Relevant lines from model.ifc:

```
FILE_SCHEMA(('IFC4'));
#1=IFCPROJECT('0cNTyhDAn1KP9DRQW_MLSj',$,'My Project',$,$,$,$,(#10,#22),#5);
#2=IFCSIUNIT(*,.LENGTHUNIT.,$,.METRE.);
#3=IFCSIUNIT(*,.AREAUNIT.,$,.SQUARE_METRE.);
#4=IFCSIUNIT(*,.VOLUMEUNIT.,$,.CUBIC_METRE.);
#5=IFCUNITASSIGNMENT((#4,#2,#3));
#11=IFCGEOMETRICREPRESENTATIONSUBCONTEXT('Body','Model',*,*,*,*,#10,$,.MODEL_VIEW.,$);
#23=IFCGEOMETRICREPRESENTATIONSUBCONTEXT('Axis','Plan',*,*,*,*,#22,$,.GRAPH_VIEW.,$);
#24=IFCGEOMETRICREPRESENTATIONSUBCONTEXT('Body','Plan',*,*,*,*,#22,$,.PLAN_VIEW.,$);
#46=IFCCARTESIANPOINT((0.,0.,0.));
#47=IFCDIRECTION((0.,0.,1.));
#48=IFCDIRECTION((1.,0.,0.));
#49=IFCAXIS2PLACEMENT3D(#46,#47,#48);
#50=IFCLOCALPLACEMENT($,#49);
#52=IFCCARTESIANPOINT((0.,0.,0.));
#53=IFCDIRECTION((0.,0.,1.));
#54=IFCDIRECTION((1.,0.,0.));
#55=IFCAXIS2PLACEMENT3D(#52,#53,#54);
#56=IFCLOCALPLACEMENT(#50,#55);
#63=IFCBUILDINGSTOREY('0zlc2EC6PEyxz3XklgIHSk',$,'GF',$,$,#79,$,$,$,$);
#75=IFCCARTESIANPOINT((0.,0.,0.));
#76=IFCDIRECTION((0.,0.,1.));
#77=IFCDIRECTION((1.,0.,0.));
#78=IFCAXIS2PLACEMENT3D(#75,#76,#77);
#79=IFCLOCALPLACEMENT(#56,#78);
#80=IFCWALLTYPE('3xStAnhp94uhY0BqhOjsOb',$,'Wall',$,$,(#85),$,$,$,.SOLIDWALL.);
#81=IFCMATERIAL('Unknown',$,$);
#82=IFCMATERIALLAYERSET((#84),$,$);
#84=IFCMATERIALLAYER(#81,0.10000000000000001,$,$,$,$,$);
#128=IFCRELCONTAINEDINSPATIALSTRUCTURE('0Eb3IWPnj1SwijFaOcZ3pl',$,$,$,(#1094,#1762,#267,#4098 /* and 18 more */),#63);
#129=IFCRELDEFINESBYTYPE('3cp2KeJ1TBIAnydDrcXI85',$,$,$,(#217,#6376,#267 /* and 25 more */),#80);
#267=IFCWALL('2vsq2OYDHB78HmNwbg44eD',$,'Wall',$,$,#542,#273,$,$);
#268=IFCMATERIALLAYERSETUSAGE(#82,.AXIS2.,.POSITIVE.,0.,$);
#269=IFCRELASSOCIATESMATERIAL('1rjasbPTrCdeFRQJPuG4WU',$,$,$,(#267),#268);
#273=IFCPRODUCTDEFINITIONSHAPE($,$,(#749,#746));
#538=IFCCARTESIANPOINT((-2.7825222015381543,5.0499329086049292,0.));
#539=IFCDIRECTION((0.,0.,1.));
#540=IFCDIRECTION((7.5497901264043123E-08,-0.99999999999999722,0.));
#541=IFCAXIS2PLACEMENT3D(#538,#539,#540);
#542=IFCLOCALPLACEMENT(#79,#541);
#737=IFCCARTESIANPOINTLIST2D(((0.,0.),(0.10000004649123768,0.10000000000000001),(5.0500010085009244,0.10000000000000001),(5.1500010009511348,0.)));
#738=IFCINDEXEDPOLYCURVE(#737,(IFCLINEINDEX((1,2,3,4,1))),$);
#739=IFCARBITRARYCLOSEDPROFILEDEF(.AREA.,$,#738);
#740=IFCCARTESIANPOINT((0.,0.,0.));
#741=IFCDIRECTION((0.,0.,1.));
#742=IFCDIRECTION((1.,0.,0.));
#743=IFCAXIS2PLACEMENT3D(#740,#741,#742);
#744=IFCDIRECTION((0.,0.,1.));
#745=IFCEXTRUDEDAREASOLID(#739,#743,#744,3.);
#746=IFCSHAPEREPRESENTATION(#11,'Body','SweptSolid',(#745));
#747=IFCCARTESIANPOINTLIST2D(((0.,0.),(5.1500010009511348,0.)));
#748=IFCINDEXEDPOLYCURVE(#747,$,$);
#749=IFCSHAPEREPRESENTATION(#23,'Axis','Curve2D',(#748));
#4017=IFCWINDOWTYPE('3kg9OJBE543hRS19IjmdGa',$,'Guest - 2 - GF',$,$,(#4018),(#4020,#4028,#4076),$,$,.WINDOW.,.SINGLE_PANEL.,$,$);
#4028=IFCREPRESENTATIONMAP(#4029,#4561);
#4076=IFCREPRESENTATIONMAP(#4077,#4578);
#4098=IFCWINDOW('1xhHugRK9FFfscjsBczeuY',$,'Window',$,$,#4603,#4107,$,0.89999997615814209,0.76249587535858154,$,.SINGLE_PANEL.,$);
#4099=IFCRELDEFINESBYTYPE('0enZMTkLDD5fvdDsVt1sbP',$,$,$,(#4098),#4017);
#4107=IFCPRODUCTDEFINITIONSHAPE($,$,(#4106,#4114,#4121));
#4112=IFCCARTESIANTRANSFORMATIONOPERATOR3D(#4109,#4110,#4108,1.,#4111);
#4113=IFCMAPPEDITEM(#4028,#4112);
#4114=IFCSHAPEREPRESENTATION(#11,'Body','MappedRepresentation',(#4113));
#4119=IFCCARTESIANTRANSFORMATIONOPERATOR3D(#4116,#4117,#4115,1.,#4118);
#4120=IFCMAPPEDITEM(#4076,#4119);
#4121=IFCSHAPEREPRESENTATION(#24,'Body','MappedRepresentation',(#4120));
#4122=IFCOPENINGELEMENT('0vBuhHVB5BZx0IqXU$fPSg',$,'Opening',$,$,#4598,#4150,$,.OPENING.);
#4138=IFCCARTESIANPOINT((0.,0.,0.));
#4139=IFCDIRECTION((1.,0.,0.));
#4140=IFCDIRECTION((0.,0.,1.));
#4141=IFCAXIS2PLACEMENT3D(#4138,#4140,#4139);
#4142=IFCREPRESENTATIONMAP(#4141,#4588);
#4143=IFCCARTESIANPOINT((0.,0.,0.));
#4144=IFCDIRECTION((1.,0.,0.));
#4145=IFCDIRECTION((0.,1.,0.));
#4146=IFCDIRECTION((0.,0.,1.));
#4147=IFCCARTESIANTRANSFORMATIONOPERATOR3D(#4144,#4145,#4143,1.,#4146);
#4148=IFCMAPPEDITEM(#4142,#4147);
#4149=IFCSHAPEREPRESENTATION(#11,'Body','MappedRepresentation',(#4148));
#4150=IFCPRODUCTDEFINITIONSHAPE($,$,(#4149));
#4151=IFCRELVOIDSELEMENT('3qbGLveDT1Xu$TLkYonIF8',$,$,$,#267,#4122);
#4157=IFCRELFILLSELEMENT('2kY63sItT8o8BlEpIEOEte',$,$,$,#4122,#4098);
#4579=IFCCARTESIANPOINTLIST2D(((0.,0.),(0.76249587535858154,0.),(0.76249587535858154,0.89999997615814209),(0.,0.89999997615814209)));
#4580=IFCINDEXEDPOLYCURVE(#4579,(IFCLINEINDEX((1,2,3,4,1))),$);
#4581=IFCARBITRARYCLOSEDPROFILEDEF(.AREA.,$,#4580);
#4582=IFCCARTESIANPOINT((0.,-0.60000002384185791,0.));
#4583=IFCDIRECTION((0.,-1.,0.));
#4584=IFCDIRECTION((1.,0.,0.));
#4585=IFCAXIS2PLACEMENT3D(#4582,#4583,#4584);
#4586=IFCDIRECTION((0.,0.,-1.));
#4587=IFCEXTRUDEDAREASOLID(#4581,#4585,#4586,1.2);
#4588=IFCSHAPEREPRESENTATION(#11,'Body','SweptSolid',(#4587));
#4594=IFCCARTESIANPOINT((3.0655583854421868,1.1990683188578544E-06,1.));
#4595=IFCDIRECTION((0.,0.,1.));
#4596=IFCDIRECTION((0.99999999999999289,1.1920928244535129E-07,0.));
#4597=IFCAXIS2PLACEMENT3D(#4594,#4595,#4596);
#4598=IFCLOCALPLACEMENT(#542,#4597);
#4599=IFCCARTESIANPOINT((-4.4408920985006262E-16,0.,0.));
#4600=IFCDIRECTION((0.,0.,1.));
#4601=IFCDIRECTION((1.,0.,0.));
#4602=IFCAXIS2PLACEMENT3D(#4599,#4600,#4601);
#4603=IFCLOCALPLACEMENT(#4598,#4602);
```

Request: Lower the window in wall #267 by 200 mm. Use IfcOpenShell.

```python
import numpy as np
import ifcopenshell
import ifcopenshell.api.geometry
import ifcopenshell.util.placement
import ifcopenshell.util.unit

model = ifcopenshell.open("model.ifc")
unit_scale = ifcopenshell.util.unit.calculate_unit_scale(model)

window = model.by_id(4098)
opening = window.FillsVoids[0].RelatingOpeningElement
dz = -0.2

shift = np.array([0.0, 0.0, dz])
# The window is placed relative to its opening, so it follows when the opening moves.
matrix = ifcopenshell.util.placement.get_local_placement(opening.ObjectPlacement)
matrix[:3, 3] += shift
ifcopenshell.api.geometry.edit_object_placement(
    model, product=opening, matrix=matrix, is_si=False, should_transform_children=True
)

print(f"moved by {dz * unit_scale:+.3f} m")

model.write("model_v2.ifc")
```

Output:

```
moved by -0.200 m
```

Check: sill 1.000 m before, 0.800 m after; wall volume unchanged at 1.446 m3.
